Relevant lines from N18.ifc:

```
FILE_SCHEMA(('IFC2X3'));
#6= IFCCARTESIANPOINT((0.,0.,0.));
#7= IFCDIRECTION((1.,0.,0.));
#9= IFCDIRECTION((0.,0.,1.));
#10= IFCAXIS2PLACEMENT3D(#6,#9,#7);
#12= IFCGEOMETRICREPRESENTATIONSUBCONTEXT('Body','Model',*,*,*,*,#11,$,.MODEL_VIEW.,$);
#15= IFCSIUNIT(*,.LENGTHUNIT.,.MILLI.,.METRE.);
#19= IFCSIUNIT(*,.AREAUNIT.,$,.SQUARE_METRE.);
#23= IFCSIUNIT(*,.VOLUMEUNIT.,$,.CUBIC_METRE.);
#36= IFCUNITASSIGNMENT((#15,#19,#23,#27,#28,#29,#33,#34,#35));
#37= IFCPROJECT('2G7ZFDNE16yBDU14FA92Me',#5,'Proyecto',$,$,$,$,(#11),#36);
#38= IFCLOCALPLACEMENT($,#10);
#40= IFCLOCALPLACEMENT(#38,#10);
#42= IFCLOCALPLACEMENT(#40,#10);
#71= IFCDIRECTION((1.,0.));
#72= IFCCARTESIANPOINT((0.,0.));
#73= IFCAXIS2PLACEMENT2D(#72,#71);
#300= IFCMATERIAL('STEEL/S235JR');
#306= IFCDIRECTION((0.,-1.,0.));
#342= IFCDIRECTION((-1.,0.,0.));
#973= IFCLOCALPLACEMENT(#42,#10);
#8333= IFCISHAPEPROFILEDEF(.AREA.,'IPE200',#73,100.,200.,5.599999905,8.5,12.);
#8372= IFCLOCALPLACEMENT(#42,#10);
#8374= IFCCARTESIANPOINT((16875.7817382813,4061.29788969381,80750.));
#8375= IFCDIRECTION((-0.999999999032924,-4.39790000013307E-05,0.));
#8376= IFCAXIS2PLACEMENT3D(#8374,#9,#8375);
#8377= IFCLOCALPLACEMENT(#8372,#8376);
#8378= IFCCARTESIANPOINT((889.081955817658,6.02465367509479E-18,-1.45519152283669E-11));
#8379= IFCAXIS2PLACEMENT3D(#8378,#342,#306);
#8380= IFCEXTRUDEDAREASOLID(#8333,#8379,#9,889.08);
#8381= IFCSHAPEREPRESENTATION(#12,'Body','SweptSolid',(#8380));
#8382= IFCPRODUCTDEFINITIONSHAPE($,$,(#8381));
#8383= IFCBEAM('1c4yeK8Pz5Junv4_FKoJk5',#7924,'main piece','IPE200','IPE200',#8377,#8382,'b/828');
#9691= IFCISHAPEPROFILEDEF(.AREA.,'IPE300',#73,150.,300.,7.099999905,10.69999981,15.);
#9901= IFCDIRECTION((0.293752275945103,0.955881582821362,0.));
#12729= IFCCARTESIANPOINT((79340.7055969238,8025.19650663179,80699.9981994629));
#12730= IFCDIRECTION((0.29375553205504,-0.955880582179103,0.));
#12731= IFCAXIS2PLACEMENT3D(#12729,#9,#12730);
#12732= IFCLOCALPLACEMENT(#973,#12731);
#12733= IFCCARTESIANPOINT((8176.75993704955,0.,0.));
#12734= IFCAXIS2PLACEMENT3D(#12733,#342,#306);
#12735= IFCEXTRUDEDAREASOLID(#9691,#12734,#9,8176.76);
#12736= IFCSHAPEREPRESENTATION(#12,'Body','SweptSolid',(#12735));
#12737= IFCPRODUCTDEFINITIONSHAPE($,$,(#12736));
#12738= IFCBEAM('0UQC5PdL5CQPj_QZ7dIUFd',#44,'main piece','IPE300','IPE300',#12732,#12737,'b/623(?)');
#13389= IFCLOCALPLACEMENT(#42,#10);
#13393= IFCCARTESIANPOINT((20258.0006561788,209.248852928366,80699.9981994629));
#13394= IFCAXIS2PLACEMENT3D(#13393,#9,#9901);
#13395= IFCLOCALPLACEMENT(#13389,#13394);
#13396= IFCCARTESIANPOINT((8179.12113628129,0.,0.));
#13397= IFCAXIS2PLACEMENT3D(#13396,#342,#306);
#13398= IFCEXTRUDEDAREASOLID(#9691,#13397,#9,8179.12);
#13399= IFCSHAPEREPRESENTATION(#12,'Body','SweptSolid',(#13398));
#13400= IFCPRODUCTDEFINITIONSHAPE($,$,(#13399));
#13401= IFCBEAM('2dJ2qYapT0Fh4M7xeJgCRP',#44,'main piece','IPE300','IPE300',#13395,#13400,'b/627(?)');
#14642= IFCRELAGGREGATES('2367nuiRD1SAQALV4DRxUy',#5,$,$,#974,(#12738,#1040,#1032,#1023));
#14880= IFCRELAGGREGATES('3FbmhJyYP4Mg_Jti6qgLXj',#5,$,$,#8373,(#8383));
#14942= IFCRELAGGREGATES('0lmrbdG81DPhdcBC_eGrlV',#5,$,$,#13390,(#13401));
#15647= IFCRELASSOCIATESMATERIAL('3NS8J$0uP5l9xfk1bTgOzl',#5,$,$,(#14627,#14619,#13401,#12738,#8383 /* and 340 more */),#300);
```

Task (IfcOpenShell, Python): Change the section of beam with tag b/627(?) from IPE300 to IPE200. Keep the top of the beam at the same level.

```python
import ifcopenshell
import ifcopenshell.util.element
import ifcopenshell.util.representation

model = ifcopenshell.open("N18.ifc")

member = model.by_guid("2dJ2qYapT0Fh4M7xeJgCRP")
source = next(p for p in model.by_type("IfcIShapeProfileDef") if p.ProfileName == "IPE200")

body = ifcopenshell.util.representation.get_representation(member, "Model", "Body")
solid = body.Items[0]
old_profile = solid.SweptArea

# Copy the section's sizes but keep this member's own profile position.
profile = ifcopenshell.util.element.copy(model, source)
# Profiles are centred, so shift by half the change in depth to hold the top.
shift = (old_profile.OverallDepth - profile.OverallDepth) / 2
x, y = old_profile.Position.Location.Coordinates
up = (0.0, 1.0)  # upwards, in the solid's own plane
location = model.createIfcCartesianPoint((x + up[0] * shift, y + up[1] * shift))
profile.Position = model.createIfcAxis2Placement2D(location, old_profile.Position.RefDirection)
solid.SweptArea = profile
if not model.get_total_inverses(old_profile):
    ifcopenshell.util.element.remove_deep2(model, old_profile)
member.Description = member.Description.replace("IPE300", "IPE200")
member.ObjectType = member.ObjectType.replace("IPE300", "IPE200")

print(solid.SweptArea)

model.write("N18_edited.ifc")
```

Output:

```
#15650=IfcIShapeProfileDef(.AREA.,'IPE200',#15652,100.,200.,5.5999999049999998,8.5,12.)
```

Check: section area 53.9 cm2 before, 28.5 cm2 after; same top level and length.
